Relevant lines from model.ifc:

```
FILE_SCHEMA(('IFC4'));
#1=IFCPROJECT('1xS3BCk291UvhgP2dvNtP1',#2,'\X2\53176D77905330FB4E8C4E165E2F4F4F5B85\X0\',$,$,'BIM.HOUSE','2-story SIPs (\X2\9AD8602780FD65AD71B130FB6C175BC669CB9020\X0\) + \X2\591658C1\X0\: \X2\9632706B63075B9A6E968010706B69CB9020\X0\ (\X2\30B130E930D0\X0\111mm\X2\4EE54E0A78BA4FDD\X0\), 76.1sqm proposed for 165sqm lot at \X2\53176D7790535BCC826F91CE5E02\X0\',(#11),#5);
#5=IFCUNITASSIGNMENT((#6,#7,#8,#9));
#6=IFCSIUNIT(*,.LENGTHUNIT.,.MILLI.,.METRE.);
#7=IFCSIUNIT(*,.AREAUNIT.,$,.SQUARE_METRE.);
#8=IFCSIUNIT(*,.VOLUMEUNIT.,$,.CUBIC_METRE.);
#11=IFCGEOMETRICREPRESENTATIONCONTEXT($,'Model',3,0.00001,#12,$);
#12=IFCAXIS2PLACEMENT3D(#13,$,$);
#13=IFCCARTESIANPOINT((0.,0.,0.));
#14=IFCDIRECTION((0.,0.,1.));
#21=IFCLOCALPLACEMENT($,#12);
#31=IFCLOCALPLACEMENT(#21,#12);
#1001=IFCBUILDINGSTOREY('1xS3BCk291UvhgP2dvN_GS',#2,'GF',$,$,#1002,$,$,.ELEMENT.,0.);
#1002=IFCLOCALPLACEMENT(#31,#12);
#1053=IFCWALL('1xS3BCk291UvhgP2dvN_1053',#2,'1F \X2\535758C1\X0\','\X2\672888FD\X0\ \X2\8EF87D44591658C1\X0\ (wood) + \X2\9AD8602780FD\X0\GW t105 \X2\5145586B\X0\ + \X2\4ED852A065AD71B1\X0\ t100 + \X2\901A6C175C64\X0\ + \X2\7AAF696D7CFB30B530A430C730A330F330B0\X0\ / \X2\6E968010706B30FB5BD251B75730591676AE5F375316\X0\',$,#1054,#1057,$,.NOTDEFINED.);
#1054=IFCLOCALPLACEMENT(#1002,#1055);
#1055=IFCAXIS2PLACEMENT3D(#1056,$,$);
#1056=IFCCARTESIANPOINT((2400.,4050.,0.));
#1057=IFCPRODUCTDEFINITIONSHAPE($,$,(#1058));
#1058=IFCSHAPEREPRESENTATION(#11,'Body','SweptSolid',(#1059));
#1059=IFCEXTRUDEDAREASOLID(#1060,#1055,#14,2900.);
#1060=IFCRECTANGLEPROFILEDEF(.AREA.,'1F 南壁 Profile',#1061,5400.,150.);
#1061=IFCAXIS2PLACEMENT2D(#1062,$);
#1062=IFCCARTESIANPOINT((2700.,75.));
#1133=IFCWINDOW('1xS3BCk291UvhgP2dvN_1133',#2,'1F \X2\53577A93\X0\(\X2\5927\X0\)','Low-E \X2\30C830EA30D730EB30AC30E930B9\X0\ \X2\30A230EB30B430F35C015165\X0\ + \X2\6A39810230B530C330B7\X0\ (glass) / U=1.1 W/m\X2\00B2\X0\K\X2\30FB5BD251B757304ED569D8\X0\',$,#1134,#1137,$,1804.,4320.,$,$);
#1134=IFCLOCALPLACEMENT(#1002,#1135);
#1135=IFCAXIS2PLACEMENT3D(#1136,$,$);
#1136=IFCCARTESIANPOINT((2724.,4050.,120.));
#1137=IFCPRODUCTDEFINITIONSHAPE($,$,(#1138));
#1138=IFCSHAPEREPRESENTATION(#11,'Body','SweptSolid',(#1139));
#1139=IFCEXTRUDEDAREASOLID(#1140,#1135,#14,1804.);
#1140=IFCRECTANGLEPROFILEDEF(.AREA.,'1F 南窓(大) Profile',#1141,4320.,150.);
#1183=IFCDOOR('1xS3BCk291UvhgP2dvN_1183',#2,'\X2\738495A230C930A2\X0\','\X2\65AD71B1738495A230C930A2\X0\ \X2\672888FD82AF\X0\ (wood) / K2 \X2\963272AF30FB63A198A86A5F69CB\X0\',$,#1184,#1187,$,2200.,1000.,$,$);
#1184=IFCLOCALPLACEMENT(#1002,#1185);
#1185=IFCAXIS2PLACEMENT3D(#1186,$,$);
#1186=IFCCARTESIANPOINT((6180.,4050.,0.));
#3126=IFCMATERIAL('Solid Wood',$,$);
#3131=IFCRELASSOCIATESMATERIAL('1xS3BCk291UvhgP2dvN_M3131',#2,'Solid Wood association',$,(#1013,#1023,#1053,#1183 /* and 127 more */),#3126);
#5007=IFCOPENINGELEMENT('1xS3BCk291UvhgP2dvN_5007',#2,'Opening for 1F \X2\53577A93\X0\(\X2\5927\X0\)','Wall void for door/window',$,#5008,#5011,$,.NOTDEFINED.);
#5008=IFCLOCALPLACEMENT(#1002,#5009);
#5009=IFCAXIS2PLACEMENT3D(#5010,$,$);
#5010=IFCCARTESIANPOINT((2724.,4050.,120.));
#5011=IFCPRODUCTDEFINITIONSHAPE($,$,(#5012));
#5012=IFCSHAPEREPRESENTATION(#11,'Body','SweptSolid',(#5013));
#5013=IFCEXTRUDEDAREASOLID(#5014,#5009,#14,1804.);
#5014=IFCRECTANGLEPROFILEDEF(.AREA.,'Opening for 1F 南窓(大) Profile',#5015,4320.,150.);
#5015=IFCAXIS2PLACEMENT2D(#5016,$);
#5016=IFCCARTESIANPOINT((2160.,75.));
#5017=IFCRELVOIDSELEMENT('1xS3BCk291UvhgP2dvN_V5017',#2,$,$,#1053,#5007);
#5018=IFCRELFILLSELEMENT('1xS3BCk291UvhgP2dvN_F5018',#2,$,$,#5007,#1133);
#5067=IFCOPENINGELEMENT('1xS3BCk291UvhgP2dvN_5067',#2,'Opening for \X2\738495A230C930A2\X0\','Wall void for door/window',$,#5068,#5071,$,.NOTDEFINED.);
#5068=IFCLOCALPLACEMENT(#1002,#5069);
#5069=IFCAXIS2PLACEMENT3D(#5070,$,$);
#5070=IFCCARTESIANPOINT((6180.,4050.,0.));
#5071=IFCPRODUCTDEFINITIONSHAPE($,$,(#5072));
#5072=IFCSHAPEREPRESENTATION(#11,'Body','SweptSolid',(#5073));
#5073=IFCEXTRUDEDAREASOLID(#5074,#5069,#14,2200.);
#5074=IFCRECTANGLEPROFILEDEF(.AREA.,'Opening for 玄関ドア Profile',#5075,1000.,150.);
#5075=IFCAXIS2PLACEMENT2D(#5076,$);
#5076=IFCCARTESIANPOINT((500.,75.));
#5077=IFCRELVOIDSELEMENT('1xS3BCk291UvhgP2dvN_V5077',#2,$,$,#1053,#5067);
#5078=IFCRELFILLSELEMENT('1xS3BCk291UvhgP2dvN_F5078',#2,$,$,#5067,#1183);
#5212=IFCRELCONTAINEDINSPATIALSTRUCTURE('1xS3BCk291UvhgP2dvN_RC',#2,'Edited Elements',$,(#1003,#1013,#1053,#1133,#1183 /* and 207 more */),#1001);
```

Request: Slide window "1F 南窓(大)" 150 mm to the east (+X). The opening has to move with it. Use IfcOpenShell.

```python
import ifcopenshell
import ifcopenshell.api.geometry
import ifcopenshell.util.placement
import ifcopenshell.util.unit

model = ifcopenshell.open("model.ifc")
unit_scale = ifcopenshell.util.unit.calculate_unit_scale(model)

window = model.by_id(1133)
opening = window.FillsVoids[0].RelatingOpeningElement
wall = opening.VoidsElements[0].RelatingBuildingElement

wall_matrix = ifcopenshell.util.placement.get_local_placement(wall.ObjectPlacement)
shift = wall_matrix[:3, 0] * 0.15 / unit_scale
before = ifcopenshell.util.placement.get_local_placement(window.ObjectPlacement)[:3, 3].copy()

# The window is not placed relative to its opening, so move both.
for product in (opening, window):
    matrix = ifcopenshell.util.placement.get_local_placement(product.ObjectPlacement)
    matrix[:3, 3] += shift
    ifcopenshell.api.geometry.edit_object_placement(model, product=product, matrix=matrix, is_si=False)

after = ifcopenshell.util.placement.get_local_placement(window.ObjectPlacement)[:3, 3]
print("window moved by", (after - before).round(3) + 0.0)

model.write("model_edited.ifc")
```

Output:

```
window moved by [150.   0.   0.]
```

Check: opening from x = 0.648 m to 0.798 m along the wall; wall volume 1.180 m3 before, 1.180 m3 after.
